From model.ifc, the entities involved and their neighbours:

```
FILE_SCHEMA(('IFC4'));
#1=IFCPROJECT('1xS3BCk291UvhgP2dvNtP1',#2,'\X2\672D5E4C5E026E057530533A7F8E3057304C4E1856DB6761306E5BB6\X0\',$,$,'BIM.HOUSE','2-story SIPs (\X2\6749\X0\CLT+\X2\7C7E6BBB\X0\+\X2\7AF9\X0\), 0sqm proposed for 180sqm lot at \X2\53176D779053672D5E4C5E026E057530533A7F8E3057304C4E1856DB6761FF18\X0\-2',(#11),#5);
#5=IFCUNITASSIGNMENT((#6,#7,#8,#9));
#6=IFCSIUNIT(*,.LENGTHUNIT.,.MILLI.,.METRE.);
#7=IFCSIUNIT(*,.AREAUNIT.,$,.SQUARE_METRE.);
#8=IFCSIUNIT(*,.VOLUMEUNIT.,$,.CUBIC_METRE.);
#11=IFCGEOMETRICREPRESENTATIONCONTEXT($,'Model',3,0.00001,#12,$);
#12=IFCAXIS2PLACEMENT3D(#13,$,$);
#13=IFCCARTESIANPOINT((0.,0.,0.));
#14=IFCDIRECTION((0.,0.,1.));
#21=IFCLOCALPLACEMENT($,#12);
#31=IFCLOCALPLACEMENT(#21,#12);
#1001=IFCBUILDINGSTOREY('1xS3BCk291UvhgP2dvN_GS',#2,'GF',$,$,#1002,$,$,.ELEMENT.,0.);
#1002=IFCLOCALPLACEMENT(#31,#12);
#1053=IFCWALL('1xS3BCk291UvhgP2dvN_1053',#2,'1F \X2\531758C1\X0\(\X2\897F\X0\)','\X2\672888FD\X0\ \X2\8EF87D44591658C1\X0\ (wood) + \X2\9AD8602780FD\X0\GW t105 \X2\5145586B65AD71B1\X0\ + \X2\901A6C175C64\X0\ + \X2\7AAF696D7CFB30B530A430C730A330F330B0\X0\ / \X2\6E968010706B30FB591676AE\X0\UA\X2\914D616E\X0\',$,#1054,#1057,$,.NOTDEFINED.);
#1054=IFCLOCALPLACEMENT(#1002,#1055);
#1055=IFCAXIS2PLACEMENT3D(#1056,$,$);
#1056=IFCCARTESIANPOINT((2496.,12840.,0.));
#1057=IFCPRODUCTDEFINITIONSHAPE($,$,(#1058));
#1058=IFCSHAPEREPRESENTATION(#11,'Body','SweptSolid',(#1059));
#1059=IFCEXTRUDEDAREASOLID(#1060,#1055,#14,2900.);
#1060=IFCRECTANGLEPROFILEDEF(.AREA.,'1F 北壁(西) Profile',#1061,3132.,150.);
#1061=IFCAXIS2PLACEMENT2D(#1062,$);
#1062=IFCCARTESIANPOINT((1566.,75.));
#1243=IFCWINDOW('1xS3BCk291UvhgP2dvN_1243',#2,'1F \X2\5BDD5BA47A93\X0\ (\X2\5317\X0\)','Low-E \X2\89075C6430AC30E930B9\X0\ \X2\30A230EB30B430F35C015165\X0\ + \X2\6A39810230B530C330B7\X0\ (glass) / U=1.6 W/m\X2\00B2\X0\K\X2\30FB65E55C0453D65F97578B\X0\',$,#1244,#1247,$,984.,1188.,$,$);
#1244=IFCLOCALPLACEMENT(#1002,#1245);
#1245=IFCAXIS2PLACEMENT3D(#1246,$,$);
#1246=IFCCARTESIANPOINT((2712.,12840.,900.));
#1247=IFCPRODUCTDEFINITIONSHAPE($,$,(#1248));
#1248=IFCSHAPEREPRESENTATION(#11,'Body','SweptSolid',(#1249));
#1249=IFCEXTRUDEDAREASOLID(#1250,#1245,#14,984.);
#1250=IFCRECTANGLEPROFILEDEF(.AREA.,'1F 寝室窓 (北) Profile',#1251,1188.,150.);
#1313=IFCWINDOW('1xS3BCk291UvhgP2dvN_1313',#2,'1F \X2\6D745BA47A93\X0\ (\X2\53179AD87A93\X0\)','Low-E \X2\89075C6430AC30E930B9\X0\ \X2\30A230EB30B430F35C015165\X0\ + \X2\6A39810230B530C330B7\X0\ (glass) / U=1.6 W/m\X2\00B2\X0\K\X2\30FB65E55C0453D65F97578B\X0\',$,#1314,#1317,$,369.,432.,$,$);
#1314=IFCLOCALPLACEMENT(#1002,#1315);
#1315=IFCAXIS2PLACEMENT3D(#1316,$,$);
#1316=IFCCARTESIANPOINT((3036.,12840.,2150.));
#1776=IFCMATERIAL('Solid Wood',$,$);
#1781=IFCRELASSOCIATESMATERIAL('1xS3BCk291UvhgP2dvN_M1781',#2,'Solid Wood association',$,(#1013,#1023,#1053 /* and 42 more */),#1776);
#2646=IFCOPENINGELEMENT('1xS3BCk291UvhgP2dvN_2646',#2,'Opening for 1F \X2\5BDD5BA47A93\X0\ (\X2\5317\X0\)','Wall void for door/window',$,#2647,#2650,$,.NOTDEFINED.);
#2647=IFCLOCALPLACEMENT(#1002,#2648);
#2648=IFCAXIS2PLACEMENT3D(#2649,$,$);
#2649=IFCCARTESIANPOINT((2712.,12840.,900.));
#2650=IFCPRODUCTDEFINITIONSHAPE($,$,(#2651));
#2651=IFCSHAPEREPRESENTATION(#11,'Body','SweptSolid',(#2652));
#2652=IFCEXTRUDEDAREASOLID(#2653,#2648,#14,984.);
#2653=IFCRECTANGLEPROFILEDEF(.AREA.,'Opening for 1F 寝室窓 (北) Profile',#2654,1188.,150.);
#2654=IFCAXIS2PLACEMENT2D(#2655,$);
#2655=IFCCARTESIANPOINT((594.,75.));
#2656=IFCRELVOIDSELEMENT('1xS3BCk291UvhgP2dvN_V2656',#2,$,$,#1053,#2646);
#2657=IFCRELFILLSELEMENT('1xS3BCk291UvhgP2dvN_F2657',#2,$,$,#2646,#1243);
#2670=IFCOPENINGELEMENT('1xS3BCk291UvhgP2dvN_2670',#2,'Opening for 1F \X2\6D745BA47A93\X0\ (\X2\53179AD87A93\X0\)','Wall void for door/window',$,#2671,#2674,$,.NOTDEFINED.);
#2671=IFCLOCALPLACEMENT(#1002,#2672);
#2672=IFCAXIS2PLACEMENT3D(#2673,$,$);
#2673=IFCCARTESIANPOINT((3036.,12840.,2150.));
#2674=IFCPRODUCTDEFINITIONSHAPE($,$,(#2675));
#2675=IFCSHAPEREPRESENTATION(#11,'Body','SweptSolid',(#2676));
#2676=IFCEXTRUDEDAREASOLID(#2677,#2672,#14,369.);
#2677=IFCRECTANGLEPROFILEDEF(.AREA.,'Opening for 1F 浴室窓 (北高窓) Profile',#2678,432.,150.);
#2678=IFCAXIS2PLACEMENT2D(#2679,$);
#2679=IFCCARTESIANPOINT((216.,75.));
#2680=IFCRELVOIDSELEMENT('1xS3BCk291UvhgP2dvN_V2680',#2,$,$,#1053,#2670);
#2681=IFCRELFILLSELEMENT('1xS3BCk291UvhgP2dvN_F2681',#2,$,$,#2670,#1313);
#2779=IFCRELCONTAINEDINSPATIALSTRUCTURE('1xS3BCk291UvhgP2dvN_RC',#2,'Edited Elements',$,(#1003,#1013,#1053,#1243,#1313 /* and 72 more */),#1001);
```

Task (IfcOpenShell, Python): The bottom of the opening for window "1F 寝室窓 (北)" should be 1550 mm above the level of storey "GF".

```python
import numpy as np
import ifcopenshell
import ifcopenshell.api.geometry
import ifcopenshell.geom
import ifcopenshell.util.element
import ifcopenshell.util.placement
import ifcopenshell.util.shape
import ifcopenshell.util.unit

model = ifcopenshell.open("model.ifc")
unit_scale = ifcopenshell.util.unit.calculate_unit_scale(model)

window = model.by_guid("1xS3BCk291UvhgP2dvN_1243")
opening = window.FillsVoids[0].RelatingOpeningElement
storey = ifcopenshell.util.element.get_container(window, ifc_class="IfcBuildingStorey")
level = ifcopenshell.util.placement.get_local_placement(storey.ObjectPlacement)[2, 3]

# The opening's origin need not be at the sill, so measure its lowest point.
shape = ifcopenshell.geom.create_shape(ifcopenshell.geom.settings(), opening)
bottom = ifcopenshell.util.shape.get_shape_bottom_elevation(shape, shape.geometry) / unit_scale
dz = level + 1.55 / unit_scale - bottom

shift = np.array([0.0, 0.0, dz])
# The window is not placed relative to its opening, so move both.
for product in (opening, window):
    matrix = ifcopenshell.util.placement.get_local_placement(product.ObjectPlacement)
    matrix[:3, 3] += shift
    ifcopenshell.api.geometry.edit_object_placement(model, product=product, matrix=matrix, is_si=False)

print(f"moved by {dz * unit_scale:+.3f} m")

model.write("model-out.ifc")
```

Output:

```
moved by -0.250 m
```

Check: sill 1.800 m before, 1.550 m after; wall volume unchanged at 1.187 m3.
